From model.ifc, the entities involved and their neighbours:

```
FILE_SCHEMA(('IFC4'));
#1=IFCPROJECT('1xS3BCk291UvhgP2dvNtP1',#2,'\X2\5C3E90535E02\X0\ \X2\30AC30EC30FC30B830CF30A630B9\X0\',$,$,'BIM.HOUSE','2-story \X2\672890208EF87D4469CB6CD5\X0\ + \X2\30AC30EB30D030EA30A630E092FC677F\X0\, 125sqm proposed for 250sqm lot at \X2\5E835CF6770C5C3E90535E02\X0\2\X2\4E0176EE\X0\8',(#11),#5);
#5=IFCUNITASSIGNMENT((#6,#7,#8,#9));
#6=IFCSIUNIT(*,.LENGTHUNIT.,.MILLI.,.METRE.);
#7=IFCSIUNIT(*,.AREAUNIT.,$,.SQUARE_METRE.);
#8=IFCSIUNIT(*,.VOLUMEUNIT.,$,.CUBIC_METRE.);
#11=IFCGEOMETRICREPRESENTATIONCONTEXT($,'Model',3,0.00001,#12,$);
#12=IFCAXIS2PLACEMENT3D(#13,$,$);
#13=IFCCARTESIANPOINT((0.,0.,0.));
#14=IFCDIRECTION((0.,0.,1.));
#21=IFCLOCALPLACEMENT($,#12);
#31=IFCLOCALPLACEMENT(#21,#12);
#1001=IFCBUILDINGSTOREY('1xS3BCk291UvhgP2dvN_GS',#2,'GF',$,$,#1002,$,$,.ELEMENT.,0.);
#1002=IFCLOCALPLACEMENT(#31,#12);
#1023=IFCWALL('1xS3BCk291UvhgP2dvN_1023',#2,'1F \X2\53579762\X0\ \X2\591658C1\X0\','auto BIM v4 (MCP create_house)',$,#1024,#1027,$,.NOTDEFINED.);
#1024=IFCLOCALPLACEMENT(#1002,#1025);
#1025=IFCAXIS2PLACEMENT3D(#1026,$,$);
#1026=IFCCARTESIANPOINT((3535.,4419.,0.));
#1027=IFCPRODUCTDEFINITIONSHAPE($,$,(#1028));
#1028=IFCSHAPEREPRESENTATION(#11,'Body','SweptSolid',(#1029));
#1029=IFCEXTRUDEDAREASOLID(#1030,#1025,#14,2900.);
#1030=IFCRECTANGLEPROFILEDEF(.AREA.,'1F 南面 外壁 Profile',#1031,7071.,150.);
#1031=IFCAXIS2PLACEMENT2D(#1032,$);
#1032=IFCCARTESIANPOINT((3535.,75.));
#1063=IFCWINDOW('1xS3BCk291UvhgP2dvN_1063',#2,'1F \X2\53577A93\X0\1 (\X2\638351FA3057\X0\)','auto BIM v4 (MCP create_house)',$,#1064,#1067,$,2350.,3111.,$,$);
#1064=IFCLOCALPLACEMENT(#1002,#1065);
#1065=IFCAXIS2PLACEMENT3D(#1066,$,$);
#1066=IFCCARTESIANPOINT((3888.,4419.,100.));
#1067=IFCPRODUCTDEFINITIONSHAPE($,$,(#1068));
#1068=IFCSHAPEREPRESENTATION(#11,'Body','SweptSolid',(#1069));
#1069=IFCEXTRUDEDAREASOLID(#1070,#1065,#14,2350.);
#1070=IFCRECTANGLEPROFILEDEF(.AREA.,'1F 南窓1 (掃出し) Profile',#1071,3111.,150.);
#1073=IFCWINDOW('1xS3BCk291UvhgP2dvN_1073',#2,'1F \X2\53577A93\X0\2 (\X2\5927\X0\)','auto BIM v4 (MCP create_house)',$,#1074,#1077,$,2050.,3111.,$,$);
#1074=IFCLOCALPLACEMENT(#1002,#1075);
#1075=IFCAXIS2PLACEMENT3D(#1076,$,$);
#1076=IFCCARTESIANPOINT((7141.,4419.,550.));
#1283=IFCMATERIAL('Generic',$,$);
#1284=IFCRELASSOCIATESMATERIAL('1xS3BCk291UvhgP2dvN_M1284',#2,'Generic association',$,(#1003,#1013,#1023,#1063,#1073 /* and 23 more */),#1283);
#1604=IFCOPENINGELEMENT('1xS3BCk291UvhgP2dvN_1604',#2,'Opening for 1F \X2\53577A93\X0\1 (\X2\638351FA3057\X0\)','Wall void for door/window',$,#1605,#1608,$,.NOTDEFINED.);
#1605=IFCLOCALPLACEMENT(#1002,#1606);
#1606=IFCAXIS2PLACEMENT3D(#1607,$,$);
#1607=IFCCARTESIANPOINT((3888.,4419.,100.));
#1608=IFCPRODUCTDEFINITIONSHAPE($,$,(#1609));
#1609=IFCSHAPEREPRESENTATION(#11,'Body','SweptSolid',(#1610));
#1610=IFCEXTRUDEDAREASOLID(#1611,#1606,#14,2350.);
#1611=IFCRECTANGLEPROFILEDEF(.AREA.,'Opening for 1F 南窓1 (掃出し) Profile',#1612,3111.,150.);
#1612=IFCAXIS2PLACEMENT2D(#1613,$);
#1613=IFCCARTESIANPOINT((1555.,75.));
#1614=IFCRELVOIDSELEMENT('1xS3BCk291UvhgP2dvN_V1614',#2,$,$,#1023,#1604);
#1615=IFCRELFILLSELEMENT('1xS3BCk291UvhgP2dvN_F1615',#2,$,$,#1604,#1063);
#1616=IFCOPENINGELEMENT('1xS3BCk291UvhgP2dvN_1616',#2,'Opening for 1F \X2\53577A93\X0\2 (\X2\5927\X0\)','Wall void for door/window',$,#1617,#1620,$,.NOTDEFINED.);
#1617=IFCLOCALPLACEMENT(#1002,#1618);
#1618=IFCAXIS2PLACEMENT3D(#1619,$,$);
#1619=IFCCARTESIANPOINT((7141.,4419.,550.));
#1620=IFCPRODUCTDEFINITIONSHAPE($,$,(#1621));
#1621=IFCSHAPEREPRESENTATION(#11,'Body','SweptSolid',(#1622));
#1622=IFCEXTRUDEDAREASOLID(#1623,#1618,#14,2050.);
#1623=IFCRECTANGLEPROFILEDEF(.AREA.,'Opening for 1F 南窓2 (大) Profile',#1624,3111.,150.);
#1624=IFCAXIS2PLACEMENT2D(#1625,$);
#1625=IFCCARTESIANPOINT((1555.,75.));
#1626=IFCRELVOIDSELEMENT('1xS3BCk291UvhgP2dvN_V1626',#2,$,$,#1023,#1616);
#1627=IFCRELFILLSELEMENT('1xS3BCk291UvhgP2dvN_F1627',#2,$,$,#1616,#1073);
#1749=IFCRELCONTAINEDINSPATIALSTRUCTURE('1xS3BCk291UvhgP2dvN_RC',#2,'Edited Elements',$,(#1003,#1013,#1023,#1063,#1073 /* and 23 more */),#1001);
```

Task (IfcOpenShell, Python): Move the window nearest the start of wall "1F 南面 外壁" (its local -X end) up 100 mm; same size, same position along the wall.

```python
import numpy as np
import ifcopenshell
import ifcopenshell.api.geometry
import ifcopenshell.util.placement
import ifcopenshell.util.unit

model = ifcopenshell.open("model.ifc")
unit_scale = ifcopenshell.util.unit.calculate_unit_scale(model)

window = model.by_guid("1xS3BCk291UvhgP2dvN_1063")
opening = window.FillsVoids[0].RelatingOpeningElement
dz = 0.1 / unit_scale

shift = np.array([0.0, 0.0, dz])
# The window is not placed relative to its opening, so move both.
for product in (opening, window):
    matrix = ifcopenshell.util.placement.get_local_placement(product.ObjectPlacement)
    matrix[:3, 3] += shift
    ifcopenshell.api.geometry.edit_object_placement(model, product=product, matrix=matrix, is_si=False)

print(f"moved by {dz * unit_scale:+.3f} m")

model.write("model_rev.ifc")
```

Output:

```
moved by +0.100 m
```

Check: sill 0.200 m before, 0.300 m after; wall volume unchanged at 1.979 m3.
